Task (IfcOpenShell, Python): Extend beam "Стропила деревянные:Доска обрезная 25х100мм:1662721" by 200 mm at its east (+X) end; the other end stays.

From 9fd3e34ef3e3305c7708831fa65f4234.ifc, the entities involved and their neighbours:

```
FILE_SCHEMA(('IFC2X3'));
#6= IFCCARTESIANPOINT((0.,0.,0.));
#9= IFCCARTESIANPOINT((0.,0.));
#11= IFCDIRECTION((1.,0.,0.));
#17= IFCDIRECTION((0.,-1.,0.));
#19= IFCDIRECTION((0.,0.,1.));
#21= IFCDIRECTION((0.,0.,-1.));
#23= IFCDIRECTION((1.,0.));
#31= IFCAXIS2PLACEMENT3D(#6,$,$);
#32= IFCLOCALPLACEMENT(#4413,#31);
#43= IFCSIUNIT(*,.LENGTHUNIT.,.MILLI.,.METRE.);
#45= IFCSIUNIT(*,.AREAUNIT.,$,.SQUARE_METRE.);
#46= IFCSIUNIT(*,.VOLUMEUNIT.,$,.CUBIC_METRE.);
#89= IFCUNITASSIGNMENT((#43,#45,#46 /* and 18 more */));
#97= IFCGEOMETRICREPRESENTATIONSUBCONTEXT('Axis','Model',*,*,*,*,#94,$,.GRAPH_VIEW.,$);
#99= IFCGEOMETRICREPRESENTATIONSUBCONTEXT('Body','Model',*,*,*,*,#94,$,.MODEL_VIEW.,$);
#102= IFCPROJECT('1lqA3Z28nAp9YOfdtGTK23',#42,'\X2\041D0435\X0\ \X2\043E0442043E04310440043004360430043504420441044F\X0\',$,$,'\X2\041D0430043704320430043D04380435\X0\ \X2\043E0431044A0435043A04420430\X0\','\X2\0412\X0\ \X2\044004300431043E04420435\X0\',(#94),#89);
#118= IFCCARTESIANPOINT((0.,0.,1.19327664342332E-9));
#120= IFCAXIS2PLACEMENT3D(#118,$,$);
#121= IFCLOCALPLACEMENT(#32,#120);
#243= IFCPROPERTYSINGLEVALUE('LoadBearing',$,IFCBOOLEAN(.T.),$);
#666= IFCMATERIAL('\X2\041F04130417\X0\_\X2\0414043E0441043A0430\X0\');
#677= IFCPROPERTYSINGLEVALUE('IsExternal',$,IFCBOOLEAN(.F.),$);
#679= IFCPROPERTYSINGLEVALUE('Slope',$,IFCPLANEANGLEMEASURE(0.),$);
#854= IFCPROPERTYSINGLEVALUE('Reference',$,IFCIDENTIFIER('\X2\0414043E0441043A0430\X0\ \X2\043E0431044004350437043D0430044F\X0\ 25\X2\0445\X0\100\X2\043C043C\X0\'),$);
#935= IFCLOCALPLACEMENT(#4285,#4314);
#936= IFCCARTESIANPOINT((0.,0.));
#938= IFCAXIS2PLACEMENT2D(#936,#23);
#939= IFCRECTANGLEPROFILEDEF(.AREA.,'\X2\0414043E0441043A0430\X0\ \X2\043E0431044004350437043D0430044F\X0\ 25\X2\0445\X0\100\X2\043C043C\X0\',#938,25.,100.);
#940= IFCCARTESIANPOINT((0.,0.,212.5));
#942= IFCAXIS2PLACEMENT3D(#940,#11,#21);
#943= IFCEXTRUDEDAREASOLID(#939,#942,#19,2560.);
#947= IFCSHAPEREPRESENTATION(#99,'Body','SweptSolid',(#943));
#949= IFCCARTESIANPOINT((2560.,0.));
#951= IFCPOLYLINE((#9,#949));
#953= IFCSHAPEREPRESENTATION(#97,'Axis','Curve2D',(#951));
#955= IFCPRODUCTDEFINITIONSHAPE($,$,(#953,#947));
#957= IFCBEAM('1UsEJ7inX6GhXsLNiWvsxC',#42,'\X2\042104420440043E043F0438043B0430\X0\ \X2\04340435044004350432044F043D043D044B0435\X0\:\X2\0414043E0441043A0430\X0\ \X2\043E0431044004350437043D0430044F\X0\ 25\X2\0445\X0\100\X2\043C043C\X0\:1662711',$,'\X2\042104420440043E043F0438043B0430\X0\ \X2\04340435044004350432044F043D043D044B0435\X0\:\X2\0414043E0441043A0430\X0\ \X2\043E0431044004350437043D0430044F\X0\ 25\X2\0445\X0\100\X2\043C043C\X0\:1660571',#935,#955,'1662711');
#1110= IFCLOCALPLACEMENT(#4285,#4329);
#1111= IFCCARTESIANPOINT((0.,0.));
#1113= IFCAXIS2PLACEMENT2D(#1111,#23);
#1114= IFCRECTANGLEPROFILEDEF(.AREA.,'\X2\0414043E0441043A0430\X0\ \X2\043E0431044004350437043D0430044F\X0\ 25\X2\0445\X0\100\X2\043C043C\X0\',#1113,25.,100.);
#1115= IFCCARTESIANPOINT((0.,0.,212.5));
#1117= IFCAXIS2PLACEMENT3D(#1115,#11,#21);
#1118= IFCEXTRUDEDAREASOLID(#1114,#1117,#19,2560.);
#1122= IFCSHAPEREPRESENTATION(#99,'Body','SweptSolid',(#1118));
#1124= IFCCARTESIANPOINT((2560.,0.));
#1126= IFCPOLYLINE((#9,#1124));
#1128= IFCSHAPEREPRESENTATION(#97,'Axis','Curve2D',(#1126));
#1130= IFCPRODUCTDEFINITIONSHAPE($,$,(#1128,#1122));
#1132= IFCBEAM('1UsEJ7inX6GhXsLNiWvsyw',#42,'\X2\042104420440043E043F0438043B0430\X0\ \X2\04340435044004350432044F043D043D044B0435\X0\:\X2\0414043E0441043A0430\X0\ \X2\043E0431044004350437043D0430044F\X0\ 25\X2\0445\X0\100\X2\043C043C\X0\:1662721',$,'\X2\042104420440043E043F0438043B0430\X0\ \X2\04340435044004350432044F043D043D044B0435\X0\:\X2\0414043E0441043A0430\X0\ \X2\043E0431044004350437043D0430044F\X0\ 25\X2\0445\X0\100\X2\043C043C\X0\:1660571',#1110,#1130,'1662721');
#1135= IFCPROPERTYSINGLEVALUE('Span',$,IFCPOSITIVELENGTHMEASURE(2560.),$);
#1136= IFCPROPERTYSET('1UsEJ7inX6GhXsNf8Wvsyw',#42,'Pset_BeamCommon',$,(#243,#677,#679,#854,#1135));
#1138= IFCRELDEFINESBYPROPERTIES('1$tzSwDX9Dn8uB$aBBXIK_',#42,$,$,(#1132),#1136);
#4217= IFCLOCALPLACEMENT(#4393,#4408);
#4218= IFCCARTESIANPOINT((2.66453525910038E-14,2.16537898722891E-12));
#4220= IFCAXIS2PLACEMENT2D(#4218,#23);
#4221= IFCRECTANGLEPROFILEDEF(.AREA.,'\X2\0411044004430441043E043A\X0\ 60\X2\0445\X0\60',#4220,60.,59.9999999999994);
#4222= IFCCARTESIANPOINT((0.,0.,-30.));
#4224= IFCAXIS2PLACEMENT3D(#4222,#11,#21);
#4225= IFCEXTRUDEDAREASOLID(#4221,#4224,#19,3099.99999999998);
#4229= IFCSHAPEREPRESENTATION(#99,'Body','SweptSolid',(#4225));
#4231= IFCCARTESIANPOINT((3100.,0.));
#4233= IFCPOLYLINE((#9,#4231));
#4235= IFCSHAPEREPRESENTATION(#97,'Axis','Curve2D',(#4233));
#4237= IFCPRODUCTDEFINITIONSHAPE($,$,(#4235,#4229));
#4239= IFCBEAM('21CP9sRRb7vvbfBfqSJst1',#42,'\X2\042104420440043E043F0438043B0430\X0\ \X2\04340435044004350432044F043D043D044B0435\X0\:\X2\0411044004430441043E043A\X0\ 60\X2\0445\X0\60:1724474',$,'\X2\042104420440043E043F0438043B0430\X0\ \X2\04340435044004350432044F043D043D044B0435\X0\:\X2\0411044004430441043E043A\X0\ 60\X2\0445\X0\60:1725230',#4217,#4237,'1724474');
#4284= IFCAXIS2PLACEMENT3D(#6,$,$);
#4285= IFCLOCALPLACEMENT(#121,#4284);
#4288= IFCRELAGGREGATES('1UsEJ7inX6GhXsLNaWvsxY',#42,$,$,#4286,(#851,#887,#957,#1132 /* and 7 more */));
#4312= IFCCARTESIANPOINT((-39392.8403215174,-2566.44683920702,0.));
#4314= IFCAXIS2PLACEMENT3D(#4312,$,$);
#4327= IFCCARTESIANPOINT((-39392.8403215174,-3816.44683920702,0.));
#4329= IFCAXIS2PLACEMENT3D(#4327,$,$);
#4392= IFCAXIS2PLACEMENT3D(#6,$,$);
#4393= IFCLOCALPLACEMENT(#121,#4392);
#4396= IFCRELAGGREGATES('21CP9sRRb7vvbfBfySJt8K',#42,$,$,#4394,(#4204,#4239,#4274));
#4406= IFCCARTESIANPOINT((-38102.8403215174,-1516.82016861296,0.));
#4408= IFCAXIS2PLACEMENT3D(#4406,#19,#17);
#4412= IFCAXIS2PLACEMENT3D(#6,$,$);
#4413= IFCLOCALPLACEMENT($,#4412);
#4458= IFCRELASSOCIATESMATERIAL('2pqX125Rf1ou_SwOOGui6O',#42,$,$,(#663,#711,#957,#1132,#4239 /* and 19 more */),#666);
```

```python
import numpy as np
import ifcopenshell
import ifcopenshell.api.pset
import ifcopenshell.util.element
import ifcopenshell.util.representation
import ifcopenshell.util.unit

model = ifcopenshell.open("9fd3e34ef3e3305c7708831fa65f4234.ifc")
unit_scale = ifcopenshell.util.unit.calculate_unit_scale(model)

member = model.by_guid("1UsEJ7inX6GhXsLNiWvsyw")
change = 0.2 / unit_scale

# The extrusion runs towards the end named, so only its depth changes.
body = ifcopenshell.util.representation.get_representation(member, "Model", "Body")
solid = body.Items[0]
old_length = solid.Depth
solid.Depth += change

# Move the axis end point with it.
axis = next(r for r in member.Representation.Representations if r.RepresentationIdentifier == "Axis").Items[0]
start, end = (np.array(p.Coordinates) for p in axis.Points)
end = end + (end - start) / np.linalg.norm(end - start) * change
point = model.createIfcCartesianPoint(end.tolist())
axis.Points = [axis.Points[0], point]

# Update the stored length and volume.
pset = model.by_id(ifcopenshell.util.element.get_pset(member, "Pset_BeamCommon", should_inherit=False)["id"])
ifcopenshell.api.pset.edit_pset(model, pset=pset, properties={
    "Span": model.create_entity("IfcPositiveLengthMeasure", solid.Depth),
})

print(f"length {old_length:g} -> {solid.Depth:g}")

model.write("9fd3e34ef3e3305c7708831fa65f4234_edited.ifc")
```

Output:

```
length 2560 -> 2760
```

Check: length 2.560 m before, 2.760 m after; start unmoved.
